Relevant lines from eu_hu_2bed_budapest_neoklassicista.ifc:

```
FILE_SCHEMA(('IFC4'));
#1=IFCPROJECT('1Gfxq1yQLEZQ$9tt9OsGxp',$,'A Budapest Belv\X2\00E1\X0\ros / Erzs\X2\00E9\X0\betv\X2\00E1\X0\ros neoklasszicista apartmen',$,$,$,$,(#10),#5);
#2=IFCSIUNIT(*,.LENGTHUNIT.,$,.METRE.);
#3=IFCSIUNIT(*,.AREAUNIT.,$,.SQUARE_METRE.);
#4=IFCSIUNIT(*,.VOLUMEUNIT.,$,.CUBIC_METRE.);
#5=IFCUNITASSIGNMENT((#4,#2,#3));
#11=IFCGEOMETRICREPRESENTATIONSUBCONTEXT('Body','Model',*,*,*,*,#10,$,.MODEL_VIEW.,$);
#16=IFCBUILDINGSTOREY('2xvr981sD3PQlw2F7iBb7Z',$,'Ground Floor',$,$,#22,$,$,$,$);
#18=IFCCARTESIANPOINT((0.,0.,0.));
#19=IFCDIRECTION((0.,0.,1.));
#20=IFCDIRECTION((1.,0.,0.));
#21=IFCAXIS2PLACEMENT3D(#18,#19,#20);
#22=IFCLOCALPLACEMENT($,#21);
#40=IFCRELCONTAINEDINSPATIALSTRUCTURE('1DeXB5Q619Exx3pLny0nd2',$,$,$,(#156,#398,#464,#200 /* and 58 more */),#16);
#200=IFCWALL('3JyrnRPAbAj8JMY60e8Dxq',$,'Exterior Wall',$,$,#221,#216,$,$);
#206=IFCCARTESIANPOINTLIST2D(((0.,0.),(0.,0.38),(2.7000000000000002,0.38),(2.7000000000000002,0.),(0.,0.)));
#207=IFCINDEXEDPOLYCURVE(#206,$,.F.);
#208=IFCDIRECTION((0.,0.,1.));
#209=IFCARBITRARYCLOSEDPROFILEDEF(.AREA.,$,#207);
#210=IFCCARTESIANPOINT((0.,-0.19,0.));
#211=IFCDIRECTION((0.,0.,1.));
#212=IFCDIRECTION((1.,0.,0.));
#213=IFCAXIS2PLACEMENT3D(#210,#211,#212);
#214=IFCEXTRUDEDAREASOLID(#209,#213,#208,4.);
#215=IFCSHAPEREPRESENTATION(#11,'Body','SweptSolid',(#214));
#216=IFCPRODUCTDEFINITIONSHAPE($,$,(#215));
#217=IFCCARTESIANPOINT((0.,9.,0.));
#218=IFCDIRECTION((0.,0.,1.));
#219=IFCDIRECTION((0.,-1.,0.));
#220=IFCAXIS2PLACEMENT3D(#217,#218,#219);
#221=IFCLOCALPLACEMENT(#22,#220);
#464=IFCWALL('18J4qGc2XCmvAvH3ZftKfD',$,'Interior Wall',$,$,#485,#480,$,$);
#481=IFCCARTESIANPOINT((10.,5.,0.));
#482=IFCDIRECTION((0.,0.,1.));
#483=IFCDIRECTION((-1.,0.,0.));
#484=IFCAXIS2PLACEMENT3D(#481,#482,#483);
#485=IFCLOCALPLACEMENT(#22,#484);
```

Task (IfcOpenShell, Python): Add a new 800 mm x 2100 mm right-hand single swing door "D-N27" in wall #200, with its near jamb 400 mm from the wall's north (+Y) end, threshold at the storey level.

```python
import numpy as np
import ifcopenshell
import ifcopenshell.api.feature
import ifcopenshell.api.geometry
import ifcopenshell.api.root
import ifcopenshell.api.spatial
import ifcopenshell.geom
import ifcopenshell.util.element
import ifcopenshell.util.placement
import ifcopenshell.util.representation
import ifcopenshell.util.shape
import ifcopenshell.util.unit

model = ifcopenshell.open("eu_hu_2bed_budapest_neoklassicista.ifc")
unit_scale = ifcopenshell.util.unit.calculate_unit_scale(model)
settings = ifcopenshell.geom.settings()


def volume(element):
    """Net volume in cubic metres, openings subtracted."""
    shape = ifcopenshell.geom.create_shape(settings, element)
    return ifcopenshell.util.shape.get_volume(shape.geometry)


wall = model.by_guid("3JyrnRPAbAj8JMY60e8Dxq")
storey = ifcopenshell.util.element.get_container(wall, ifc_class="IfcBuildingStorey")
context = ifcopenshell.util.representation.get_context(model, "Model", "Body", "MODEL_VIEW")
before = volume(wall)

width, height, from_end, sill = 0.8, 2.1, 0.4, 0.0  # metres

# The wall runs along its own X axis, and the end named is its -X end.
wall_shape = ifcopenshell.geom.create_shape(settings, wall)
x, y, z = ifcopenshell.util.shape.get_vertices(wall_shape.geometry).T
start = x.min() + from_end
face, thickness = float(y.min()), float(y.max() - y.min())
wall_matrix = ifcopenshell.util.placement.get_local_placement(wall.ObjectPlacement)
level = ifcopenshell.util.placement.get_local_placement(storey.ObjectPlacement)[2, 3]


def in_wall(x, y):
    """Placement at x, y metres in the wall's axes, at sill height."""
    matrix = wall_matrix.copy()
    matrix[:, 3] = wall_matrix @ np.array([x / unit_scale, y / unit_scale, 0.0, 1.0])
    matrix[2, 3] = level + sill / unit_scale
    return matrix


# Opening: a box that overshoots both wall faces by 50 mm.
opening = ifcopenshell.api.root.create_entity(model, ifc_class="IfcOpeningElement", predefined_type="OPENING")
box = ifcopenshell.api.geometry.add_wall_representation(
    model, context=context, length=width, height=height, thickness=thickness + 0.1
)
ifcopenshell.api.geometry.assign_representation(model, product=opening, representation=box)
ifcopenshell.api.geometry.edit_object_placement(model, product=opening, matrix=in_wall(start, face - 0.05), is_si=False)
ifcopenshell.api.feature.add_feature(model, feature=opening, element=wall)

door = ifcopenshell.api.root.create_entity(model, ifc_class="IfcDoor", name="D-N27", predefined_type="DOOR")
door.OverallWidth, door.OverallHeight = width / unit_scale, height / unit_scale
door.OperationType = "SINGLE_SWING_RIGHT"
body = ifcopenshell.api.geometry.add_door_representation(
    model,
    context=context,
    overall_width=door.OverallWidth,
    overall_height=door.OverallHeight,
    operation_type="SINGLE_SWING_RIGHT",
    lining_properties={"LiningDepth": thickness / unit_scale, "ThresholdDepth": thickness / unit_scale},
)
ifcopenshell.api.geometry.assign_representation(model, product=door, representation=body)
ifcopenshell.api.spatial.assign_container(model, products=[door], relating_structure=storey)
ifcopenshell.api.feature.add_filling(model, opening=opening, element=door)

# The lining spans the wall, so the door starts at the wall face.
ifcopenshell.api.geometry.edit_object_placement(model, product=door, matrix=in_wall(start, face), is_si=False)

after = volume(wall)

print(f"wall volume {before:.3f} -> {after:.3f} m3")

model.write("eu_hu_2bed_budapest_neoklassicista_rev.ifc")
```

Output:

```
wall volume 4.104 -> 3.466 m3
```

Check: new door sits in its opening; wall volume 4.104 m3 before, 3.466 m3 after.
